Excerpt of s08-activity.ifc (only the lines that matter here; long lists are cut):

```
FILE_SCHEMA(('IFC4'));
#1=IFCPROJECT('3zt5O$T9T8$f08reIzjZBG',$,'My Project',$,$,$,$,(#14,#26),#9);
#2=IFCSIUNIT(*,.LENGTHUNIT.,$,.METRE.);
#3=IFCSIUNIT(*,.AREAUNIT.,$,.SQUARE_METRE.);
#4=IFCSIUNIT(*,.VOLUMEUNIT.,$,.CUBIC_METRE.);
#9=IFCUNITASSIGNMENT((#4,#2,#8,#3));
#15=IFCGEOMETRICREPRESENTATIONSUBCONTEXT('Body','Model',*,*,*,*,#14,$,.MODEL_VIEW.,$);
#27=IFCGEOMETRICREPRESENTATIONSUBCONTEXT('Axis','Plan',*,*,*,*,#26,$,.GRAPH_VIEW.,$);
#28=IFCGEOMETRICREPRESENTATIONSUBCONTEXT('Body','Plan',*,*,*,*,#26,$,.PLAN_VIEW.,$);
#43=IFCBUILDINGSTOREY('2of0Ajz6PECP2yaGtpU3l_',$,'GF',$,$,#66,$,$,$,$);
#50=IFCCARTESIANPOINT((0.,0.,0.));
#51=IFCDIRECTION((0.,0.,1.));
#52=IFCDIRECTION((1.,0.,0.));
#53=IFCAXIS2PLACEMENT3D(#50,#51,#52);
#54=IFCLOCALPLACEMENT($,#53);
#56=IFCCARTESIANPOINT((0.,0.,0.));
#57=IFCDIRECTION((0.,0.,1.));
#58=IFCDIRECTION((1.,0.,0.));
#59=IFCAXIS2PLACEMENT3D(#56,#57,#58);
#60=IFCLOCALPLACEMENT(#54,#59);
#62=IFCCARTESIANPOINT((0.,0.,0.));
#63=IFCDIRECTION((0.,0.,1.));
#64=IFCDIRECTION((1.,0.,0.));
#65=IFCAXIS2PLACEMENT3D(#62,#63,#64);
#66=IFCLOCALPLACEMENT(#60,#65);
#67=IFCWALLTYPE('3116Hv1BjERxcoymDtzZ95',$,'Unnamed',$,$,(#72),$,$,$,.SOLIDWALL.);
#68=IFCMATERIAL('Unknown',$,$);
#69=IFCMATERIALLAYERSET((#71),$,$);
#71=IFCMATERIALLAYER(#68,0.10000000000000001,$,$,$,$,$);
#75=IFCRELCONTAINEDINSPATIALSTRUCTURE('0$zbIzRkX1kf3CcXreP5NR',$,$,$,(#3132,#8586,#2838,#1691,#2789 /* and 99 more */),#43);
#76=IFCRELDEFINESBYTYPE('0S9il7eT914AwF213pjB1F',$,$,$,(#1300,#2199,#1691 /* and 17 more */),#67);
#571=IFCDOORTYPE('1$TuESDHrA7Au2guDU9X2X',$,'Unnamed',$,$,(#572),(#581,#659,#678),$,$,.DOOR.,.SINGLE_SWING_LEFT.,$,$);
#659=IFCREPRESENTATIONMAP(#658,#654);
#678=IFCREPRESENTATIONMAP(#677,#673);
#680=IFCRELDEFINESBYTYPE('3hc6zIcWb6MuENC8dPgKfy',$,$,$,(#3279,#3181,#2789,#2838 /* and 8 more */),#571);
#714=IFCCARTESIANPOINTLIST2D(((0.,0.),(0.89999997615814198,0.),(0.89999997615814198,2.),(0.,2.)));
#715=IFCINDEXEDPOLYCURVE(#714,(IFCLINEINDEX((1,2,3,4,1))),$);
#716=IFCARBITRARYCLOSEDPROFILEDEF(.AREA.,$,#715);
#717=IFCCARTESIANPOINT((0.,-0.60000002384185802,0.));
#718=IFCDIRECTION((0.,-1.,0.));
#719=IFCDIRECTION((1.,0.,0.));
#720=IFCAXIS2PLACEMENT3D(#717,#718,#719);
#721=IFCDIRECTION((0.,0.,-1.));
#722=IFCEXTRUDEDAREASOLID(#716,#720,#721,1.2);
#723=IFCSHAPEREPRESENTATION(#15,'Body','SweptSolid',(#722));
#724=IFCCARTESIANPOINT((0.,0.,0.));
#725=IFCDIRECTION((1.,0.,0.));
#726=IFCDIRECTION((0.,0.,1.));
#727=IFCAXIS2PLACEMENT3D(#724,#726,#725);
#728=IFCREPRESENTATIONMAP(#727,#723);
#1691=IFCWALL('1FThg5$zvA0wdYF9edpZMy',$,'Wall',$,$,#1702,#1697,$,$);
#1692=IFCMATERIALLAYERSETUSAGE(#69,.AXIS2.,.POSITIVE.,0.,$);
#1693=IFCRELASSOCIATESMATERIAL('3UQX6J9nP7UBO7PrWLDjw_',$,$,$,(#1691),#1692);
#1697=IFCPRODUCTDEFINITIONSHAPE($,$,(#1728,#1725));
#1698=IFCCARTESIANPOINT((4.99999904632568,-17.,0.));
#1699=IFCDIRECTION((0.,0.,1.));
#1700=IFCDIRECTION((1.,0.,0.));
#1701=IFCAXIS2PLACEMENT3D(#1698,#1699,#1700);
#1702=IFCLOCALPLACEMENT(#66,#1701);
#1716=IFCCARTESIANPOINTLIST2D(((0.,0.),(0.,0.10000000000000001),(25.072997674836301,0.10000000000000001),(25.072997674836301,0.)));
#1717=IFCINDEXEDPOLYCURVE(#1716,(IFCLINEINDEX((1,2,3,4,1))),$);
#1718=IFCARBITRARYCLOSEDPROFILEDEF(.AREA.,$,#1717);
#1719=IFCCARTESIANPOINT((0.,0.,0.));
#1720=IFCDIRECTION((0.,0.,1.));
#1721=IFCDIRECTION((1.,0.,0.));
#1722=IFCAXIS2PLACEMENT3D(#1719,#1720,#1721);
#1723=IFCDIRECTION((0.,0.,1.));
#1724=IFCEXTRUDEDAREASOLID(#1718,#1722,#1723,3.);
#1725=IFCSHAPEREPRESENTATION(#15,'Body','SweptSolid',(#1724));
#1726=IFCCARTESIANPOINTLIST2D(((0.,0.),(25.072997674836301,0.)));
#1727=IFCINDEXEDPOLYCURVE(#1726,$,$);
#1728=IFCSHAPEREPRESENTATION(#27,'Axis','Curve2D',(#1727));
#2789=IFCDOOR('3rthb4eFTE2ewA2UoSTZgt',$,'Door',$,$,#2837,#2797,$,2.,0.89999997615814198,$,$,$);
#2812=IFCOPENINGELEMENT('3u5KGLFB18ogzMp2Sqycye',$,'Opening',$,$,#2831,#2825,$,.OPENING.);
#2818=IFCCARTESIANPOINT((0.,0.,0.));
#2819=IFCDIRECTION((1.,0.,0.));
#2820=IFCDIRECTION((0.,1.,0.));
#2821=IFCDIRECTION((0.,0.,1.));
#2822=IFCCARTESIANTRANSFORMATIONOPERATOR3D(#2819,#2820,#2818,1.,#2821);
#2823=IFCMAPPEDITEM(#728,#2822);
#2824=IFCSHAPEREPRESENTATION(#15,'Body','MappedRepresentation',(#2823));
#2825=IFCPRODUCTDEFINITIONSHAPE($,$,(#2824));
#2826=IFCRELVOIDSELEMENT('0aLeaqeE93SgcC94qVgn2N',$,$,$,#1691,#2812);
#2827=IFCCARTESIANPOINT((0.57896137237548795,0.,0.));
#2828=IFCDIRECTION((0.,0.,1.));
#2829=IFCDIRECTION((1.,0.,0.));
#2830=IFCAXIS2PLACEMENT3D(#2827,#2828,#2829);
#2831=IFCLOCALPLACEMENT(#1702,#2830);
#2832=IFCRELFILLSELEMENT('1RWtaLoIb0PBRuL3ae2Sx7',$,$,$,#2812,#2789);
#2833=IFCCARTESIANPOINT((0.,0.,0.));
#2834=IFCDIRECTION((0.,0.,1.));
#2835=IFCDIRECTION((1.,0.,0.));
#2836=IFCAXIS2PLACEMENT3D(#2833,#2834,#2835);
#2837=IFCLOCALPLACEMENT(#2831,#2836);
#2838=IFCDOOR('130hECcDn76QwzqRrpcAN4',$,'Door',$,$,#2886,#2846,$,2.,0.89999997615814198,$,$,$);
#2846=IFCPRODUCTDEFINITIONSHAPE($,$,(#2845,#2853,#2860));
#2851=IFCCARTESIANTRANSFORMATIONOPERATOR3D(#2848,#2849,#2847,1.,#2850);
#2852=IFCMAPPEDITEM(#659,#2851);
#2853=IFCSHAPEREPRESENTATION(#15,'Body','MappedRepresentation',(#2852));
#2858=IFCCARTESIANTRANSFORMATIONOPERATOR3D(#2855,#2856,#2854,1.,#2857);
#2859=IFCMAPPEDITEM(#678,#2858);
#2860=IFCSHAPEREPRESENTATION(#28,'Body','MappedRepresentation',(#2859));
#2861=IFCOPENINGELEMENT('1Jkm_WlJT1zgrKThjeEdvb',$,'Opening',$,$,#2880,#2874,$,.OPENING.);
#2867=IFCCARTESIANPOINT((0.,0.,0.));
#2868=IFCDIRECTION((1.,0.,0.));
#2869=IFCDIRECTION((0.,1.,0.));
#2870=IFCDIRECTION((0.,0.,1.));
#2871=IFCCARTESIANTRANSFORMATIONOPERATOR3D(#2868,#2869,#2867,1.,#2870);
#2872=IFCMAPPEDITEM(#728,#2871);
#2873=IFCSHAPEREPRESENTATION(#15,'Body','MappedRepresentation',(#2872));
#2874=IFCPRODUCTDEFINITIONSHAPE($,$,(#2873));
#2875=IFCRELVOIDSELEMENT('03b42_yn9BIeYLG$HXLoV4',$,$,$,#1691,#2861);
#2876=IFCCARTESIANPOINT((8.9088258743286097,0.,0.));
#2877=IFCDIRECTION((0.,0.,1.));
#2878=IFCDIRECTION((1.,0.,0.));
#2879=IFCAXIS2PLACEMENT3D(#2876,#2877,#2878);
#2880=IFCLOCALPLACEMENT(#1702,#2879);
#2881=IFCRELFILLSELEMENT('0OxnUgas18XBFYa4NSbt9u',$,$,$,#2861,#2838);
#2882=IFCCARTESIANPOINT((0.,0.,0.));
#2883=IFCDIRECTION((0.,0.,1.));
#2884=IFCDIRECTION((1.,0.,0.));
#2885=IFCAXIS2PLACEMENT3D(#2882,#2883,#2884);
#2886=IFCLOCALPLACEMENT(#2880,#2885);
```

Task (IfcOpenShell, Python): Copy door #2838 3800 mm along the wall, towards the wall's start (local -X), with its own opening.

```python
import ifcopenshell
import ifcopenshell.api.feature
import ifcopenshell.api.geometry
import ifcopenshell.api.root
import ifcopenshell.geom
import ifcopenshell.util.element
import ifcopenshell.util.placement
import ifcopenshell.util.shape

model = ifcopenshell.open("s08-activity.ifc")
settings = ifcopenshell.geom.settings()


def volume(element):
    """Net volume in cubic metres, openings subtracted."""
    shape = ifcopenshell.geom.create_shape(settings, element)
    return ifcopenshell.util.shape.get_volume(shape.geometry)


door = model.by_guid("130hECcDn76QwzqRrpcAN4")
opening = door.FillsVoids[0].RelatingOpeningElement
wall = opening.VoidsElements[0].RelatingBuildingElement
before = volume(wall)
shift = ifcopenshell.util.placement.get_local_placement(wall.ObjectPlacement)[:3, 0] * -3.8

# copy_class copies the void relationship, type, container and properties, but no geometry.
new_opening = ifcopenshell.api.root.copy_class(model, product=opening)
new_opening.Representation = ifcopenshell.util.element.copy_deep(
    model, opening.Representation, exclude=["IfcGeometricRepresentationContext", "IfcRepresentationMap"]
)
new_door = ifcopenshell.api.root.copy_class(model, product=door)
new_door.Representation = ifcopenshell.util.element.copy_deep(
    model, door.Representation, exclude=["IfcGeometricRepresentationContext", "IfcRepresentationMap"]
)
ifcopenshell.api.feature.add_filling(model, opening=new_opening, element=new_door)

for old, new in ((opening, new_opening), (door, new_door)):
    matrix = ifcopenshell.util.placement.get_local_placement(old.ObjectPlacement)
    matrix[:3, 3] += shift
    ifcopenshell.api.geometry.edit_object_placement(model, product=new, matrix=matrix, is_si=False)

after = volume(wall)

print(f"wall volume {before:.3f} -> {after:.3f} m3")

model.write("s08-activity_v2.ifc")
```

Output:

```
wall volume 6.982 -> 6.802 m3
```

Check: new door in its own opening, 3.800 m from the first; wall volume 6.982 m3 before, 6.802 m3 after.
